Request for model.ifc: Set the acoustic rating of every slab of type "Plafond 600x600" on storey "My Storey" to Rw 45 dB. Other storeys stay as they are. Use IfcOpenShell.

First a look at what the model holds.

```python
import ifcopenshell
import ifcopenshell.util.element

model = ifcopenshell.open("model.ifc")
print(model.schema)
storey = next(s for s in model.by_type("IfcBuildingStorey") if s.Name == "My Storey")
slabs = [e for e in ifcopenshell.util.element.get_decomposition(storey) if e.is_a("IfcSlab")]
seen = {}
for e in slabs:
    element_type = ifcopenshell.util.element.get_type(e)
    key = (element_type.Name if element_type != e and element_type else None, ifcopenshell.util.element.get_pset(e, "Pset_SlabCommon", "AcousticRating"))
    seen[key] = seen.get(key, 0) + 1
for (name, value), count in sorted(seen.items(), key=str):
    print(count, "x", name, "|", value)
```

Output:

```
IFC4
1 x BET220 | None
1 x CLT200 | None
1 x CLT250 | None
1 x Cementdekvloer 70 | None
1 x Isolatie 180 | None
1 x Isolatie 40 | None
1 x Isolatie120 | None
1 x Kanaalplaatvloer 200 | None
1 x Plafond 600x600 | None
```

```python
import ifcopenshell
import ifcopenshell.api.pset
import ifcopenshell.util.element

model = ifcopenshell.open("model.ifc")

storey = next(s for s in model.by_type("IfcBuildingStorey") if s.Name == "My Storey")
slabs = [e for e in ifcopenshell.util.element.get_decomposition(storey) if e.is_a("IfcSlab")]

count = 0
for e in slabs:
    element_type = ifcopenshell.util.element.get_type(e)
    if element_type in (None, e) or element_type.Name != "Plafond 600x600":
        continue
    # add_pset returns the element's existing set when there is one.
    pset = ifcopenshell.api.pset.add_pset(model, product=e, name="Pset_SlabCommon")
    ifcopenshell.api.pset.edit_pset(model, pset=pset, properties={"AcousticRating": "Rw 45 dB"})
    count += 1

print(count, "slabs updated")

model.write("model_updated.ifc")
```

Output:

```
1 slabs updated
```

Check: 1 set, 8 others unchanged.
